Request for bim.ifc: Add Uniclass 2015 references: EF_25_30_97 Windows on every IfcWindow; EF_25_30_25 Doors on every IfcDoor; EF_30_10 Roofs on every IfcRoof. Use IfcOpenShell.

First a look at what the model holds.

```python
import ifcopenshell

model = ifcopenshell.open("bim.ifc")
print(model.schema)
print("classifications:", [c.Name for c in model.by_type("IfcClassification")])
for ifc_class in ("IfcDoor", "IfcRoof", "IfcStair", "IfcWall", "IfcWindow"):
    print(ifc_class, len(model.by_type(ifc_class)))
```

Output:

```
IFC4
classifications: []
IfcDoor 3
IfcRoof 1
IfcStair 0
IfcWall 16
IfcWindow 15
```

```python
import ifcopenshell
import ifcopenshell.api.classification

model = ifcopenshell.open("bim.ifc")

system = ifcopenshell.api.classification.add_classification(model, classification="Uniclass 2015")

codes = {
    "IfcWindow": ("EF_25_30_97", "Windows"),
    "IfcDoor": ("EF_25_30_25", "Doors"),
    "IfcRoof": ("EF_30_10", "Roofs"),
}
for ifc_class, (code, name) in codes.items():
    products = model.by_type(ifc_class)
    ifcopenshell.api.classification.add_reference(
        model, products=products, classification=system, identification=code, name=name
    )
    print(code, len(products))

model.write("bim-out.ifc")
```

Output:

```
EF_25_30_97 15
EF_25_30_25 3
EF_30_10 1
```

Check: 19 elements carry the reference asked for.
